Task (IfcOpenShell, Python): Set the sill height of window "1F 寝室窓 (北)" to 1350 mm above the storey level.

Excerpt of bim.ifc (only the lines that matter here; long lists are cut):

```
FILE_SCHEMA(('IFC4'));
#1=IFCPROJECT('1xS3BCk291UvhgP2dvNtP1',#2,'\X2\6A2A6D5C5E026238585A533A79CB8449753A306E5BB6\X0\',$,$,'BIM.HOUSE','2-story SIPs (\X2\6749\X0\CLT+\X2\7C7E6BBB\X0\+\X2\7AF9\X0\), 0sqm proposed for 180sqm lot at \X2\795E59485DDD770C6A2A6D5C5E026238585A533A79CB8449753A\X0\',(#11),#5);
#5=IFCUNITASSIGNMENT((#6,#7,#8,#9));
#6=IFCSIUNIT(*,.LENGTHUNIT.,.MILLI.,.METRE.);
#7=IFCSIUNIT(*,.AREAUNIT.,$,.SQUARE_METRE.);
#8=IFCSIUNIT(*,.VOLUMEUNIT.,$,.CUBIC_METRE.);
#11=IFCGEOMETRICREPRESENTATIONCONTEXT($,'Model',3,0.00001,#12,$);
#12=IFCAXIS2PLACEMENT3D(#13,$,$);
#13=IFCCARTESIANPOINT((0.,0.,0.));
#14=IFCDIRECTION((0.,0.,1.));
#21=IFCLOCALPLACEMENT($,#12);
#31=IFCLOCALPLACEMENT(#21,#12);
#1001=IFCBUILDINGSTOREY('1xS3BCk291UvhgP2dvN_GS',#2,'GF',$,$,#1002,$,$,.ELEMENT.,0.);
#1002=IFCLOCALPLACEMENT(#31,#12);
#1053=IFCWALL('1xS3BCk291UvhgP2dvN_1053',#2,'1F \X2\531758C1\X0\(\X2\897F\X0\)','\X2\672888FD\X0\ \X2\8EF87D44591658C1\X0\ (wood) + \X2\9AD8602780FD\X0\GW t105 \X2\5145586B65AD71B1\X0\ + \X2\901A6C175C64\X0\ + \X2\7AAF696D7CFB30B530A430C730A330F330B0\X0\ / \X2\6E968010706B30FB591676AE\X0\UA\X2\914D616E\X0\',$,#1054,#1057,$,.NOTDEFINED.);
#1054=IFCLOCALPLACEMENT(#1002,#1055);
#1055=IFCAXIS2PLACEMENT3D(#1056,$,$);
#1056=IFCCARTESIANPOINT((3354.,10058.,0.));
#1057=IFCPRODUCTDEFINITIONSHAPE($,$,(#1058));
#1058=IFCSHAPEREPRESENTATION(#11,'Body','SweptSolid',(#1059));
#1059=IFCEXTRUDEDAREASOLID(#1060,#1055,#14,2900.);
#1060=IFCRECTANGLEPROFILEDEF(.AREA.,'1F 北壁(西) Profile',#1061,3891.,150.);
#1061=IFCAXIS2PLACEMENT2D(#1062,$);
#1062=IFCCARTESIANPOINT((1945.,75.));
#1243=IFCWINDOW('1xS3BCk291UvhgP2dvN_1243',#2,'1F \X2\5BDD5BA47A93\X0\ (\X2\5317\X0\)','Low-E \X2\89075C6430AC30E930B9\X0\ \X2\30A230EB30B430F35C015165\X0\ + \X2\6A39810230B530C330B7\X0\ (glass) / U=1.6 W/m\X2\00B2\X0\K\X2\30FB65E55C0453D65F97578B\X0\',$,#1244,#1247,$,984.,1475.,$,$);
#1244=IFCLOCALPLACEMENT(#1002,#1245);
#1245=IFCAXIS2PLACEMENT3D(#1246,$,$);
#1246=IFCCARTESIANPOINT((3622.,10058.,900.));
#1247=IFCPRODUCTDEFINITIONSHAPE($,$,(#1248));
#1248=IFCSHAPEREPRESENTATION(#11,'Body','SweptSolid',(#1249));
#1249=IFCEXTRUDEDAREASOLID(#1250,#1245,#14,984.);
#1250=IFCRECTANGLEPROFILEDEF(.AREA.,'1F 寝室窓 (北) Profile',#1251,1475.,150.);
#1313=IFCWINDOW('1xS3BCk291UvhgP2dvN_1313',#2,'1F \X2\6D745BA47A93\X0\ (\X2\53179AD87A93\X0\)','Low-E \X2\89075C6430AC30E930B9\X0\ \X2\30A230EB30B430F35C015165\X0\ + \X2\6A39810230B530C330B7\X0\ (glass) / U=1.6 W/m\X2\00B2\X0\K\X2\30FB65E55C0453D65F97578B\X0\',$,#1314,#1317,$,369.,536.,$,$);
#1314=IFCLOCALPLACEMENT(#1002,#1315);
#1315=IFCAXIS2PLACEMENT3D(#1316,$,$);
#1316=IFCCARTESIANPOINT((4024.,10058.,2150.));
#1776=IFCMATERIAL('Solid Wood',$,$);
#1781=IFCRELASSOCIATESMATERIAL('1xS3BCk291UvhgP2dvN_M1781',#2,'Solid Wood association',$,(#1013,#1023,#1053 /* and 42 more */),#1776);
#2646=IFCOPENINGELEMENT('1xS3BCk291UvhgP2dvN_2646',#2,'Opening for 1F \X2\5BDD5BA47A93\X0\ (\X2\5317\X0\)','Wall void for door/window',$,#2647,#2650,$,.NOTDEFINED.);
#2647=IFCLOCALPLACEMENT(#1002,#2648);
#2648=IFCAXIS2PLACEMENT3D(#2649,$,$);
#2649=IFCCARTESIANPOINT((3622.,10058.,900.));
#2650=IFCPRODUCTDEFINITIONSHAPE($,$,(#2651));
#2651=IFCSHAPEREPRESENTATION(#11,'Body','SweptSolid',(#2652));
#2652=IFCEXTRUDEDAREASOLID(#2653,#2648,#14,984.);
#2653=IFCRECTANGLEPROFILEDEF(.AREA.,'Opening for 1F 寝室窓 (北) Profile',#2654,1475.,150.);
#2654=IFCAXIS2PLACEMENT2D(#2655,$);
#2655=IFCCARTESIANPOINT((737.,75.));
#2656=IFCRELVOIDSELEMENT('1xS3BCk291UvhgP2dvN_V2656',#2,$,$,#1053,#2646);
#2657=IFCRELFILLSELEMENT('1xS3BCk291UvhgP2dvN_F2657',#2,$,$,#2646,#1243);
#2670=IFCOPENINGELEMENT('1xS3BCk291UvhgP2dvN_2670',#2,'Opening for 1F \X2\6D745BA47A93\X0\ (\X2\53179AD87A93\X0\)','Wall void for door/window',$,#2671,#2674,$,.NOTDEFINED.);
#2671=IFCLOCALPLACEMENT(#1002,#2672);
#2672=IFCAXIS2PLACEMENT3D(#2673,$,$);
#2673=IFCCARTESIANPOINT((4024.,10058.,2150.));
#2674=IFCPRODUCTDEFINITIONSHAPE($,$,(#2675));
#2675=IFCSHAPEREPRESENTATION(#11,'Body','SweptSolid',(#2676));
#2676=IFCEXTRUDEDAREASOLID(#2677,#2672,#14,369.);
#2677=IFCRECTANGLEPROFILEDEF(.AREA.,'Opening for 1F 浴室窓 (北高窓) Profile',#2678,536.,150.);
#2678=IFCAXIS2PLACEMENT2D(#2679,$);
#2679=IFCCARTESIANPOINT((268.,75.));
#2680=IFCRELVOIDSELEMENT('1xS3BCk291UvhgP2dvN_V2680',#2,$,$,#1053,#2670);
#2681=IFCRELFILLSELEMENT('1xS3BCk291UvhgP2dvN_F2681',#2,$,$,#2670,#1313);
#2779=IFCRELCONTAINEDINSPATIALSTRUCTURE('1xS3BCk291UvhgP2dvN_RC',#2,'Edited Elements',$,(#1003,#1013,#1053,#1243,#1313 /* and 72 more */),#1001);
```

```python
import numpy as np
import ifcopenshell
import ifcopenshell.api.geometry
import ifcopenshell.geom
import ifcopenshell.util.element
import ifcopenshell.util.placement
import ifcopenshell.util.shape
import ifcopenshell.util.unit

model = ifcopenshell.open("bim.ifc")
unit_scale = ifcopenshell.util.unit.calculate_unit_scale(model)

window = model.by_id(1243)
opening = window.FillsVoids[0].RelatingOpeningElement
storey = ifcopenshell.util.element.get_container(window, ifc_class="IfcBuildingStorey")
level = ifcopenshell.util.placement.get_local_placement(storey.ObjectPlacement)[2, 3]

# The opening's origin need not be at the sill, so measure its lowest point.
shape = ifcopenshell.geom.create_shape(ifcopenshell.geom.settings(), opening)
bottom = ifcopenshell.util.shape.get_shape_bottom_elevation(shape, shape.geometry) / unit_scale
dz = level + 1.35 / unit_scale - bottom

shift = np.array([0.0, 0.0, dz])
# The window is not placed relative to its opening, so move both.
for product in (opening, window):
    matrix = ifcopenshell.util.placement.get_local_placement(product.ObjectPlacement)
    matrix[:3, 3] += shift
    ifcopenshell.api.geometry.edit_object_placement(model, product=product, matrix=matrix, is_si=False)

print(f"moved by {dz * unit_scale:+.3f} m")

model.write("bim_rev.ifc")
```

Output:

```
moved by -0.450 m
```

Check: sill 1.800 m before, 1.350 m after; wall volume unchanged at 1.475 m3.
